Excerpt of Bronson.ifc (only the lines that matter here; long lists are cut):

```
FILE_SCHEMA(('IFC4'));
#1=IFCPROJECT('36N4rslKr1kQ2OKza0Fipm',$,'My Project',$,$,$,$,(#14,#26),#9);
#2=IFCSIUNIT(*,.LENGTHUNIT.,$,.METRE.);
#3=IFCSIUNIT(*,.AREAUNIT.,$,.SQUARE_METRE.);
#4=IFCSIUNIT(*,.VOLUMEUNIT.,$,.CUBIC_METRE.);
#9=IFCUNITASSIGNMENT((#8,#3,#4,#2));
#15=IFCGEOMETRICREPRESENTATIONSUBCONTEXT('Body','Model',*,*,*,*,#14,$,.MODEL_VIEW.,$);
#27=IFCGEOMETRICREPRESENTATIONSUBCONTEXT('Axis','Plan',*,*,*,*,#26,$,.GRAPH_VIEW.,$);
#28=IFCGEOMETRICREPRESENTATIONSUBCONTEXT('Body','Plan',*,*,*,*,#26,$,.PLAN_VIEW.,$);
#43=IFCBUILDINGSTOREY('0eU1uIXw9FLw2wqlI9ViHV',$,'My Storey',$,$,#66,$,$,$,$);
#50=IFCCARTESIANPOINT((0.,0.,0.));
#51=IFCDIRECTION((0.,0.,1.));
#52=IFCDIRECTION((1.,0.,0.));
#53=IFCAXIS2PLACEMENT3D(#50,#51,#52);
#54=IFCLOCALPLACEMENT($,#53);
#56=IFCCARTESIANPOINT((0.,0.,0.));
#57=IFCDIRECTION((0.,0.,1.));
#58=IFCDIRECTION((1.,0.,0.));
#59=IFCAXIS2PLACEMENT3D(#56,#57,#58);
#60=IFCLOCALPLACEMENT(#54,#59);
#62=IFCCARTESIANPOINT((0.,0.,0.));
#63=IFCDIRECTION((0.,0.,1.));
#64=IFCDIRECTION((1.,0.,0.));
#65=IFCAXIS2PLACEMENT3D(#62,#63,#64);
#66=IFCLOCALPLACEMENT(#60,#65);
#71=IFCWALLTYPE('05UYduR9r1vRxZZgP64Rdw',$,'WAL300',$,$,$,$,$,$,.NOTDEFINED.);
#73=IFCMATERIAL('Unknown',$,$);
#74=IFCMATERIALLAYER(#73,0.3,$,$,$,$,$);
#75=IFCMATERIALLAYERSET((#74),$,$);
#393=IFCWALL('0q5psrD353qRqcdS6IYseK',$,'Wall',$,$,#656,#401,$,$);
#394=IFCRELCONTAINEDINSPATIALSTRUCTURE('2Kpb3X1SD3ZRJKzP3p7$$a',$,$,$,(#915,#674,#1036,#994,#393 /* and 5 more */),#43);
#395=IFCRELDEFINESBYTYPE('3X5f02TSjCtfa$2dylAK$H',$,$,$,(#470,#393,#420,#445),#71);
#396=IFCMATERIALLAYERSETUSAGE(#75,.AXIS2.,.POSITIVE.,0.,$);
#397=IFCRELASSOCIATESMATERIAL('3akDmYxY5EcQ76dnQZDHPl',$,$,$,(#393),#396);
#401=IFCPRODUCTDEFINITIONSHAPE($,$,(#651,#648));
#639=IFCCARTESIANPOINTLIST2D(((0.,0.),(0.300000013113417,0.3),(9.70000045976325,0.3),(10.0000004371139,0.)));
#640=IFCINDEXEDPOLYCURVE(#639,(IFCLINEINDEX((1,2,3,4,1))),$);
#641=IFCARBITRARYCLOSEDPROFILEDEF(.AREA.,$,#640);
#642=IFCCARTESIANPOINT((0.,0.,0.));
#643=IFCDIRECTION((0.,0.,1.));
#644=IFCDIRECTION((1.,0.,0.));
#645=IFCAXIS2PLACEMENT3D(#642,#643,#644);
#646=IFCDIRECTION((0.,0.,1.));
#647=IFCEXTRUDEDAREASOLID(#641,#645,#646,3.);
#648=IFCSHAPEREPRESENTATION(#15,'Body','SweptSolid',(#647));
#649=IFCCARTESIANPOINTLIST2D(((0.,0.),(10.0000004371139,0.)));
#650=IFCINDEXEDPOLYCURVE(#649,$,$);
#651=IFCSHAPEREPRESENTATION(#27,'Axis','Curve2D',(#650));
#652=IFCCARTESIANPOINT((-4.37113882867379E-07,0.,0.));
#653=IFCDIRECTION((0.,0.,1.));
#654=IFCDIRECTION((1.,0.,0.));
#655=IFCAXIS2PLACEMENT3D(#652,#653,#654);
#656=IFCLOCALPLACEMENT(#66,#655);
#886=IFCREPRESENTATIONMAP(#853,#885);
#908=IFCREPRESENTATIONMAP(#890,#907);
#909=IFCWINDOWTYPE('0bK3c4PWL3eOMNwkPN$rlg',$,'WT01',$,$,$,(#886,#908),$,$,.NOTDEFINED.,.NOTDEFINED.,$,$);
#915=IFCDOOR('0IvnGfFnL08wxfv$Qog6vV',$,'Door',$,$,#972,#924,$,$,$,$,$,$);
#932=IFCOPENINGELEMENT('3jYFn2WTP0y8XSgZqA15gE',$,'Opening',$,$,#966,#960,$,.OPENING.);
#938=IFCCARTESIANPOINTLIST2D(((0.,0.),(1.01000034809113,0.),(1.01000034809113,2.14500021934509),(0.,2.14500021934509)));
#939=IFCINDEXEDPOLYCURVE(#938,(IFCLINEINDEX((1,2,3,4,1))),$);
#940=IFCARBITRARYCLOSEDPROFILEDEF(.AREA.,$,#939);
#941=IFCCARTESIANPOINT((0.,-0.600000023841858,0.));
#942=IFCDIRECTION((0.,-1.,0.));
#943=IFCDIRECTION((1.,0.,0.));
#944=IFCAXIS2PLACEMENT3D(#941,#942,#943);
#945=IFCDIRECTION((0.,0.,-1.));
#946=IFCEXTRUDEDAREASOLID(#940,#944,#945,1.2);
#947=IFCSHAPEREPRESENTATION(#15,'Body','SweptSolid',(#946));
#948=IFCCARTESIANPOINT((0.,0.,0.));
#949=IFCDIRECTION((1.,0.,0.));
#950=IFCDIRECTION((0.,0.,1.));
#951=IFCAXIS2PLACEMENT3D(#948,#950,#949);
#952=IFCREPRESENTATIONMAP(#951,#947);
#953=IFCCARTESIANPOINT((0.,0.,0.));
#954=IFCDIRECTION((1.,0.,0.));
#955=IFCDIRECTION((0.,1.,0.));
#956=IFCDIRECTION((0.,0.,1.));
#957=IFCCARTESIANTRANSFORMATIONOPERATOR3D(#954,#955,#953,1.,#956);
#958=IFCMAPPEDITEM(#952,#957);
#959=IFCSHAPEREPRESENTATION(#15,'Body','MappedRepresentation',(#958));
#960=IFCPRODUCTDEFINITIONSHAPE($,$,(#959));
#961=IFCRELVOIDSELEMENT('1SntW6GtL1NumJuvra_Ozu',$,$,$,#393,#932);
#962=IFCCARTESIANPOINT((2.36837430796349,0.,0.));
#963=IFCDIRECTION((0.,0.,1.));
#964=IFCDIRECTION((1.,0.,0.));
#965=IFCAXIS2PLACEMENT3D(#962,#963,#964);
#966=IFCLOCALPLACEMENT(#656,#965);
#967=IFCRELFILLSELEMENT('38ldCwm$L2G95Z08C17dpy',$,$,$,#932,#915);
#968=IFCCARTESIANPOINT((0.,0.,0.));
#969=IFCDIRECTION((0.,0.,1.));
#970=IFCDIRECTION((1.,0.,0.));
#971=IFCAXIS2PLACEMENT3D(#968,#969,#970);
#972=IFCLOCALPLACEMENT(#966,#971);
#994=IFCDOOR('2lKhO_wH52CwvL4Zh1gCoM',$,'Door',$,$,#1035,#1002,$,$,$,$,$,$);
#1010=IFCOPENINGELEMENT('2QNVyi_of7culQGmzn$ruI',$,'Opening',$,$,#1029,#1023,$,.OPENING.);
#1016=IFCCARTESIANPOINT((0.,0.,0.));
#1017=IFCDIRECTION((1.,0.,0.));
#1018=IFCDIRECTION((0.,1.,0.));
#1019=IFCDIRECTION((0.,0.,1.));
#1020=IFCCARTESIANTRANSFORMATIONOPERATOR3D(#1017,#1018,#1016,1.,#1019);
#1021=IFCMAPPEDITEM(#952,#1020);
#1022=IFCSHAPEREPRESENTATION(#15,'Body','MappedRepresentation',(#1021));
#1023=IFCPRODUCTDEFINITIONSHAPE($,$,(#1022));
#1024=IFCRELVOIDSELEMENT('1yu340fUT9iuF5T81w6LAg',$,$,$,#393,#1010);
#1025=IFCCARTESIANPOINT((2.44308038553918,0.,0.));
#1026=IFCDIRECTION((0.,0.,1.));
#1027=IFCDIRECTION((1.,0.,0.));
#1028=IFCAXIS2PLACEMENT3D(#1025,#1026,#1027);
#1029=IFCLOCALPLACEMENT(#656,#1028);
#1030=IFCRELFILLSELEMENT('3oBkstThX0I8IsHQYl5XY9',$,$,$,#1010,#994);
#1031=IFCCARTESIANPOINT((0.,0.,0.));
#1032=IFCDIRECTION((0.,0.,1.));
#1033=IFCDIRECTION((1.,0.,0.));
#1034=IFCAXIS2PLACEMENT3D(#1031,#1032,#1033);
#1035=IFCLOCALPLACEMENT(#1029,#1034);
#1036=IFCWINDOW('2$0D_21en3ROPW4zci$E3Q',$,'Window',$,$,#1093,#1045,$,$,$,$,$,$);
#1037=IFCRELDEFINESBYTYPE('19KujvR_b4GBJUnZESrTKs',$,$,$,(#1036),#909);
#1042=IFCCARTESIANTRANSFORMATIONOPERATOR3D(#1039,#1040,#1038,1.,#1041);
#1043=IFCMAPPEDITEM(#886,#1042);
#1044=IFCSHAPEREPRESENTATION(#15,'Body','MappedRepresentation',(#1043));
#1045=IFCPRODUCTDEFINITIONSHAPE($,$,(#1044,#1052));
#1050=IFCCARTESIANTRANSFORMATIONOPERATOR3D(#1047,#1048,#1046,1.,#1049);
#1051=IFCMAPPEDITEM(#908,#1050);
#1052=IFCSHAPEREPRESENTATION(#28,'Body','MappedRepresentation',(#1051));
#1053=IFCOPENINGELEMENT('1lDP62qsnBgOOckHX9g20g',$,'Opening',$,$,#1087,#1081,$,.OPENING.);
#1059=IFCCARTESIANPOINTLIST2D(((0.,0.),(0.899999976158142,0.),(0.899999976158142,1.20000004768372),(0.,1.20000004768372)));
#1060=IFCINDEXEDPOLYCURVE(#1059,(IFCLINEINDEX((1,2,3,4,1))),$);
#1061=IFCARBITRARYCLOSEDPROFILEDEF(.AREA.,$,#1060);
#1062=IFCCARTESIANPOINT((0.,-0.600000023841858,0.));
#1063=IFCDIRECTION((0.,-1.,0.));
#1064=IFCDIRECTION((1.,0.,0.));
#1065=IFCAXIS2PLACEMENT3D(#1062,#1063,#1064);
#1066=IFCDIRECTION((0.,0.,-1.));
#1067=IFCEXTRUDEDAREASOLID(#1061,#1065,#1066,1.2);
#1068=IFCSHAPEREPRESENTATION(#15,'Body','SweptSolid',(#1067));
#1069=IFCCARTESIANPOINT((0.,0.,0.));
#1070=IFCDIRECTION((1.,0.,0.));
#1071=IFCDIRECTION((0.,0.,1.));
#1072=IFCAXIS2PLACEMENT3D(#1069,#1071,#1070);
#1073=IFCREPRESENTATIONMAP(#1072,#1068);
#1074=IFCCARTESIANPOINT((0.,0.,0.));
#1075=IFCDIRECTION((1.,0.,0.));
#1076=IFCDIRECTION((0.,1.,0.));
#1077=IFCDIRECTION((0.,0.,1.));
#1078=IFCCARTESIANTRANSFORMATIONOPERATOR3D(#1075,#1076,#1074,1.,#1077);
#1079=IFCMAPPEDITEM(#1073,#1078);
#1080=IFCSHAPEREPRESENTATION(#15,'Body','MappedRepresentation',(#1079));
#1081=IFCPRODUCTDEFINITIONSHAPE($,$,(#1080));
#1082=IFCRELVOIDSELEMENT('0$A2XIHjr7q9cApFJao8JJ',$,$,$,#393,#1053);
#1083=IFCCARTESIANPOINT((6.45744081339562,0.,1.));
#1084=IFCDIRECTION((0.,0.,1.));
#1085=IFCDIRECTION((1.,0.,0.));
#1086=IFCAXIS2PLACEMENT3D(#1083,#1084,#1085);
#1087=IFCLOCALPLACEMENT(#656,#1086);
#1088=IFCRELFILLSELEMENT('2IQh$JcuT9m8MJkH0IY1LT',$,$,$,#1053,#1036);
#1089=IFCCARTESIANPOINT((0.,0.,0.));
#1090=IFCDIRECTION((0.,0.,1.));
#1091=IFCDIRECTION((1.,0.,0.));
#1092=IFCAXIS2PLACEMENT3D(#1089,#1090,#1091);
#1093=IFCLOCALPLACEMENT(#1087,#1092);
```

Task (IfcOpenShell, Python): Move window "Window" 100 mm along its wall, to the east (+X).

```python
import ifcopenshell
import ifcopenshell.api.geometry
import ifcopenshell.util.placement

model = ifcopenshell.open("Bronson.ifc")

window = model.by_guid("2$0D_21en3ROPW4zci$E3Q")
opening = window.FillsVoids[0].RelatingOpeningElement
wall = opening.VoidsElements[0].RelatingBuildingElement

wall_matrix = ifcopenshell.util.placement.get_local_placement(wall.ObjectPlacement)
shift = wall_matrix[:3, 0] * 0.1
before = ifcopenshell.util.placement.get_local_placement(window.ObjectPlacement)[:3, 3].copy()

# The window is placed relative to its opening, so it follows when the opening moves.
matrix = ifcopenshell.util.placement.get_local_placement(opening.ObjectPlacement)
matrix[:3, 3] += shift
ifcopenshell.api.geometry.edit_object_placement(
    model, product=opening, matrix=matrix, is_si=False, should_transform_children=True
)

after = ifcopenshell.util.placement.get_local_placement(window.ObjectPlacement)[:3, 3]
print("window moved by", (after - before).round(3) + 0.0)

model.write("Bronson-out.ifc")
```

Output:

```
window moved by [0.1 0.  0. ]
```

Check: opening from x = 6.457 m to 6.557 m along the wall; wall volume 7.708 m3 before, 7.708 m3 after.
